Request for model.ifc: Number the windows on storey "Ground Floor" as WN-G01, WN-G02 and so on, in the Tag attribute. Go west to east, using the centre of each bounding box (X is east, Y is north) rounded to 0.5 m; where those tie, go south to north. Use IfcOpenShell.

First a look at what the model holds.

```python
import ifcopenshell
import ifcopenshell.util.element
import ifcopenshell.util.placement

model = ifcopenshell.open("model.ifc")
print(model.schema)
storey = next(s for s in model.by_type("IfcBuildingStorey") if s.Name == "Ground Floor")
windows = [e for e in ifcopenshell.util.element.get_decomposition(storey) if e.is_a("IfcWindow")]
for e in sorted(windows, key=lambda e: e.id()):
    origin = ifcopenshell.util.placement.get_local_placement(e.ObjectPlacement)[:3, 3]
    print(e.id(), e.Tag, e.Name, origin.round(2) + 0.0, sep=" | ")
```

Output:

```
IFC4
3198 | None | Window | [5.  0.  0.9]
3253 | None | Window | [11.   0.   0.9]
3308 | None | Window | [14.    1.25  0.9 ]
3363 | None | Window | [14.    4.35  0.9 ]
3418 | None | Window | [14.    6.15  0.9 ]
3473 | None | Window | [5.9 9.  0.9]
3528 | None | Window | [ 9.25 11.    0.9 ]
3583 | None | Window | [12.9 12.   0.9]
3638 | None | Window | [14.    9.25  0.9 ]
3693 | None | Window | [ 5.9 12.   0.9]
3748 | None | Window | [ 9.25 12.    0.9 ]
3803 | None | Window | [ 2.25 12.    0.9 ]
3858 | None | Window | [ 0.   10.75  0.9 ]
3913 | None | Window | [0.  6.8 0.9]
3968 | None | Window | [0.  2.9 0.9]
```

```python
import ifcopenshell
import ifcopenshell.geom
import ifcopenshell.util.element
import ifcopenshell.util.shape

model = ifcopenshell.open("model.ifc")
settings = ifcopenshell.geom.settings()
settings.set("use-world-coords", True)


def centre(element):
    shape = ifcopenshell.geom.create_shape(settings, element)
    return ifcopenshell.util.shape.get_bbox_centroid(shape.geometry)


storey = next(s for s in model.by_type("IfcBuildingStorey") if s.Name == "Ground Floor")
windows = [e for e in ifcopenshell.util.element.get_decomposition(storey) if e.is_a("IfcWindow")]

# Insertion points can sit at a corner or the storey origin, so sort by the geometry (in metres).
centres = {e: centre(e) for e in windows}
windows.sort(key=lambda e: (round(centres[e][0] / 0.5), centres[e][1]))

for i, e in enumerate(windows, start=1):
    number = f"WN-G{i:02d}"
    e.Tag = number
    print(e.id(), number)

model.write("model-out.ifc")
```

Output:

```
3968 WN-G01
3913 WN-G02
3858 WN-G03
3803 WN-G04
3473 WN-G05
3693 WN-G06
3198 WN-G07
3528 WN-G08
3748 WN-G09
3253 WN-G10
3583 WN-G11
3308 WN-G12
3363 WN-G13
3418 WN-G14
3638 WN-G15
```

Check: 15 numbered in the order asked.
